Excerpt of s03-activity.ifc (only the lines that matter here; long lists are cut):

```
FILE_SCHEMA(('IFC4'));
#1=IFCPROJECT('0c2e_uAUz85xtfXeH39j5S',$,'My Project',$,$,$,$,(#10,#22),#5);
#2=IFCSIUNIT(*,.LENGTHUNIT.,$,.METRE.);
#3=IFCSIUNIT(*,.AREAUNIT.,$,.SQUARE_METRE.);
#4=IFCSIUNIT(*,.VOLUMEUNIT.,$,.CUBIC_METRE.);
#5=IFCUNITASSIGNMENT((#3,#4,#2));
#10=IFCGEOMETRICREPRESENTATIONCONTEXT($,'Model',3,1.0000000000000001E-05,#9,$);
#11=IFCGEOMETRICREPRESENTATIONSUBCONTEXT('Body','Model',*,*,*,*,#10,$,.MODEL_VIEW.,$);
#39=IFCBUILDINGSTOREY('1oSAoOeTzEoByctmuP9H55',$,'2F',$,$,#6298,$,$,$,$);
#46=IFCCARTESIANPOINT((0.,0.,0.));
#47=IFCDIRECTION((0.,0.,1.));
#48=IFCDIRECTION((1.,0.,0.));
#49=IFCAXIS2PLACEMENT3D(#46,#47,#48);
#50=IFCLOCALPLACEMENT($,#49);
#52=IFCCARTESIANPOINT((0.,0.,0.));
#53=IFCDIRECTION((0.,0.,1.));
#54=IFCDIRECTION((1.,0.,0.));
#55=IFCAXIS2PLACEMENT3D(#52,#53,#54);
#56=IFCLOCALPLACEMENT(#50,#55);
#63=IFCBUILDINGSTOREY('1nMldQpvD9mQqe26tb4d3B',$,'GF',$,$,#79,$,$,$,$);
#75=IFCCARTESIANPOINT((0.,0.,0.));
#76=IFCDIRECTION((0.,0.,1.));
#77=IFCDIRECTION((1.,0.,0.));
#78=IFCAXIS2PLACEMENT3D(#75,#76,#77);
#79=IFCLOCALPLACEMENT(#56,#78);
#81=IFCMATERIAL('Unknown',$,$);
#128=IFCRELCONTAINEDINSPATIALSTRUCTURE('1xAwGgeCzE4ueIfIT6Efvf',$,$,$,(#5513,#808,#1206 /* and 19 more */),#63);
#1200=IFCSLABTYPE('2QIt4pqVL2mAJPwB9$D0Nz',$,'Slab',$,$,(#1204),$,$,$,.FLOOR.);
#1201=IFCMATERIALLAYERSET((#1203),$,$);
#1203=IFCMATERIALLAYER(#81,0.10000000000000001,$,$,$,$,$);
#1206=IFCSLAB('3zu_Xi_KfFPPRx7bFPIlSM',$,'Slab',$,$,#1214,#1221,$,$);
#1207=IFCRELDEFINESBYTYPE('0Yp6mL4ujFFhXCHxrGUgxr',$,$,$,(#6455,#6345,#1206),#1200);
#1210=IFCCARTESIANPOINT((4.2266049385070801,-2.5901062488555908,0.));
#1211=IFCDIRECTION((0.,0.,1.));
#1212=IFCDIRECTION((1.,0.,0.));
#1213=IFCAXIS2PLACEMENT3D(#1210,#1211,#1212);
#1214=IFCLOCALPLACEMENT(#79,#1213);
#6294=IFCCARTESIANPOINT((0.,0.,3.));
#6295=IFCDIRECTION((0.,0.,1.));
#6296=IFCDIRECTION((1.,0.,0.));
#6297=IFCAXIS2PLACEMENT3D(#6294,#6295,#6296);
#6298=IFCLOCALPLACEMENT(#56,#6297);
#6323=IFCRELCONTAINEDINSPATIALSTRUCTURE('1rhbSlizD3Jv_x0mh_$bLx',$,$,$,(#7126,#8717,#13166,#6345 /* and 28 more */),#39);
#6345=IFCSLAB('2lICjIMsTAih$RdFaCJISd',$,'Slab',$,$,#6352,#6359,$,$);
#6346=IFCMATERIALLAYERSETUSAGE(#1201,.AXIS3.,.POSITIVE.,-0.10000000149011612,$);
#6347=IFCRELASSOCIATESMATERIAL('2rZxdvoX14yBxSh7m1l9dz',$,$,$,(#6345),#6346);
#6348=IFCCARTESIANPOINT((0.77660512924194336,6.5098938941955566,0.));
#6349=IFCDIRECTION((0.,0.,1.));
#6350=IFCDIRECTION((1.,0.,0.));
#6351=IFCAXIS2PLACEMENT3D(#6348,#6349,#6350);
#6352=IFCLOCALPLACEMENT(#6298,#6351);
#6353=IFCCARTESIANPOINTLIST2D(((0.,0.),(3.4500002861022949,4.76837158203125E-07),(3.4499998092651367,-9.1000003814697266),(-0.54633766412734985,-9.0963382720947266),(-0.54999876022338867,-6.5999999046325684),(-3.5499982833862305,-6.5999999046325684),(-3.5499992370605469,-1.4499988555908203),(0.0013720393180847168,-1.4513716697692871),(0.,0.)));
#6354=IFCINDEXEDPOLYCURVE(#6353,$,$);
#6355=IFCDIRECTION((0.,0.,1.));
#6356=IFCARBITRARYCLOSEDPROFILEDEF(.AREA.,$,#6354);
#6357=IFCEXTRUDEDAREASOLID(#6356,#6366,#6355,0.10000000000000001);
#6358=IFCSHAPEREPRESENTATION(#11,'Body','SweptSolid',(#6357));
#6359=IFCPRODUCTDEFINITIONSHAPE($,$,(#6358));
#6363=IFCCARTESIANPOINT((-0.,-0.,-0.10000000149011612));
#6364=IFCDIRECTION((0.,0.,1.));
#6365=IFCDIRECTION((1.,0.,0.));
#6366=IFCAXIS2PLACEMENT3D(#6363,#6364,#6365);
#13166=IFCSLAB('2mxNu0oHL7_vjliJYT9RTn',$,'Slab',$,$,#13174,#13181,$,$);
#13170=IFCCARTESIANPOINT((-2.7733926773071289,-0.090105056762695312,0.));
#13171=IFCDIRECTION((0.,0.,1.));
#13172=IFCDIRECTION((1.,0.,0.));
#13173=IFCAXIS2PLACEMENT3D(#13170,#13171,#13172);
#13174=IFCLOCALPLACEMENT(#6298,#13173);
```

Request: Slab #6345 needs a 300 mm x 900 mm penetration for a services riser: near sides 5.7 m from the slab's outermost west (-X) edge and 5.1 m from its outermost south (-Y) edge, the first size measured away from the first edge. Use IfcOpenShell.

```python
import numpy as np
import ifcopenshell
import ifcopenshell.api.feature
import ifcopenshell.api.geometry
import ifcopenshell.api.root
import ifcopenshell.geom
import ifcopenshell.util.placement
import ifcopenshell.util.representation
import ifcopenshell.util.shape
import ifcopenshell.util.unit

model = ifcopenshell.open("s03-activity.ifc")
unit_scale = ifcopenshell.util.unit.calculate_unit_scale(model)
settings = ifcopenshell.geom.settings()


def volume(element):
    """Net volume in cubic metres, openings subtracted."""
    shape = ifcopenshell.geom.create_shape(settings, element)
    return ifcopenshell.util.shape.get_volume(shape.geometry)


slab = model.by_id(6345)
before = volume(slab)

# Extent in the slab's own axes, in metres. The edges named are its -X and -Y sides.
slab_shape = ifcopenshell.geom.create_shape(settings, slab)
vertices = ifcopenshell.util.shape.get_vertices(slab_shape.geometry)
x_min, y_min, bottom = vertices.min(axis=0)
top = vertices[:, 2].max()

opening = ifcopenshell.api.root.create_entity(model, ifc_class="IfcOpeningElement", name="Services riser opening", predefined_type="OPENING")
context = ifcopenshell.util.representation.get_context(model, "Model", "Body", "MODEL_VIEW")
width, depth = 0.3, 0.9
outline = [(0.0, 0.0), (width, 0.0), (width, depth), (0.0, depth), (0.0, 0.0)]
# Overshoot both faces by 50 mm so the cut is clean.
shape = ifcopenshell.api.geometry.add_slab_representation(
    model, context=context, depth=top - bottom + 0.1, polyline=outline
)
ifcopenshell.api.geometry.assign_representation(model, product=opening, representation=shape)

matrix = ifcopenshell.util.placement.get_local_placement(slab.ObjectPlacement)
matrix[:, 3] = matrix @ np.append(np.array([x_min + 5.7, y_min + 5.1, bottom - 0.05]) / unit_scale, 1.0)
ifcopenshell.api.geometry.edit_object_placement(model, product=opening, matrix=matrix, is_si=False)
ifcopenshell.api.feature.add_feature(model, feature=opening, element=slab)

after = volume(slab)

print(f"slab volume {before:.3f} -> {after:.3f} m3")

model.write("s03-activity_edited.ifc")
```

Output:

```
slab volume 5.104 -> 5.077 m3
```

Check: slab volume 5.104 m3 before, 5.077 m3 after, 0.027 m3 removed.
